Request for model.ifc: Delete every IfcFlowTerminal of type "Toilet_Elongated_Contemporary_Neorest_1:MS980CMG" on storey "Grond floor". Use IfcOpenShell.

First a look at what the model holds.

```python
import ifcopenshell
import ifcopenshell.util.element

model = ifcopenshell.open("model.ifc")
print(model.schema)
storey = next(s for s in model.by_type("IfcBuildingStorey") if s.Name == "Grond floor")
terminals = [e for e in ifcopenshell.util.element.get_decomposition(storey) if e.is_a("IfcFlowTerminal")]
seen = {}
for e in terminals:
    element_type = ifcopenshell.util.element.get_type(e)
    name = element_type.Name if element_type not in (None, e) else None
    seen[name] = seen.get(name, 0) + 1
for name, count in sorted(seen.items(), key=str):
    print(count, "x", name)
```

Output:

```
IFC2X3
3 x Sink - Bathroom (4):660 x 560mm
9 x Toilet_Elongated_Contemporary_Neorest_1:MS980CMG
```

```python
import ifcopenshell
import ifcopenshell.api.root
import ifcopenshell.util.element

model = ifcopenshell.open("model.ifc")

storey = next(s for s in model.by_type("IfcBuildingStorey") if s.Name == "Grond floor")
terminals = [e for e in ifcopenshell.util.element.get_decomposition(storey) if e.is_a("IfcFlowTerminal")]
targets = [e for e in terminals if (t := ifcopenshell.util.element.get_type(e)) not in (None, e) and t.Name == "Toilet_Elongated_Contemporary_Neorest_1:MS980CMG"]

for e in targets:
    ifcopenshell.api.root.remove_product(model, product=e)
print(len(targets), "removed")

model.write("model_updated.ifc")
```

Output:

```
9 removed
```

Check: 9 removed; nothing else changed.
